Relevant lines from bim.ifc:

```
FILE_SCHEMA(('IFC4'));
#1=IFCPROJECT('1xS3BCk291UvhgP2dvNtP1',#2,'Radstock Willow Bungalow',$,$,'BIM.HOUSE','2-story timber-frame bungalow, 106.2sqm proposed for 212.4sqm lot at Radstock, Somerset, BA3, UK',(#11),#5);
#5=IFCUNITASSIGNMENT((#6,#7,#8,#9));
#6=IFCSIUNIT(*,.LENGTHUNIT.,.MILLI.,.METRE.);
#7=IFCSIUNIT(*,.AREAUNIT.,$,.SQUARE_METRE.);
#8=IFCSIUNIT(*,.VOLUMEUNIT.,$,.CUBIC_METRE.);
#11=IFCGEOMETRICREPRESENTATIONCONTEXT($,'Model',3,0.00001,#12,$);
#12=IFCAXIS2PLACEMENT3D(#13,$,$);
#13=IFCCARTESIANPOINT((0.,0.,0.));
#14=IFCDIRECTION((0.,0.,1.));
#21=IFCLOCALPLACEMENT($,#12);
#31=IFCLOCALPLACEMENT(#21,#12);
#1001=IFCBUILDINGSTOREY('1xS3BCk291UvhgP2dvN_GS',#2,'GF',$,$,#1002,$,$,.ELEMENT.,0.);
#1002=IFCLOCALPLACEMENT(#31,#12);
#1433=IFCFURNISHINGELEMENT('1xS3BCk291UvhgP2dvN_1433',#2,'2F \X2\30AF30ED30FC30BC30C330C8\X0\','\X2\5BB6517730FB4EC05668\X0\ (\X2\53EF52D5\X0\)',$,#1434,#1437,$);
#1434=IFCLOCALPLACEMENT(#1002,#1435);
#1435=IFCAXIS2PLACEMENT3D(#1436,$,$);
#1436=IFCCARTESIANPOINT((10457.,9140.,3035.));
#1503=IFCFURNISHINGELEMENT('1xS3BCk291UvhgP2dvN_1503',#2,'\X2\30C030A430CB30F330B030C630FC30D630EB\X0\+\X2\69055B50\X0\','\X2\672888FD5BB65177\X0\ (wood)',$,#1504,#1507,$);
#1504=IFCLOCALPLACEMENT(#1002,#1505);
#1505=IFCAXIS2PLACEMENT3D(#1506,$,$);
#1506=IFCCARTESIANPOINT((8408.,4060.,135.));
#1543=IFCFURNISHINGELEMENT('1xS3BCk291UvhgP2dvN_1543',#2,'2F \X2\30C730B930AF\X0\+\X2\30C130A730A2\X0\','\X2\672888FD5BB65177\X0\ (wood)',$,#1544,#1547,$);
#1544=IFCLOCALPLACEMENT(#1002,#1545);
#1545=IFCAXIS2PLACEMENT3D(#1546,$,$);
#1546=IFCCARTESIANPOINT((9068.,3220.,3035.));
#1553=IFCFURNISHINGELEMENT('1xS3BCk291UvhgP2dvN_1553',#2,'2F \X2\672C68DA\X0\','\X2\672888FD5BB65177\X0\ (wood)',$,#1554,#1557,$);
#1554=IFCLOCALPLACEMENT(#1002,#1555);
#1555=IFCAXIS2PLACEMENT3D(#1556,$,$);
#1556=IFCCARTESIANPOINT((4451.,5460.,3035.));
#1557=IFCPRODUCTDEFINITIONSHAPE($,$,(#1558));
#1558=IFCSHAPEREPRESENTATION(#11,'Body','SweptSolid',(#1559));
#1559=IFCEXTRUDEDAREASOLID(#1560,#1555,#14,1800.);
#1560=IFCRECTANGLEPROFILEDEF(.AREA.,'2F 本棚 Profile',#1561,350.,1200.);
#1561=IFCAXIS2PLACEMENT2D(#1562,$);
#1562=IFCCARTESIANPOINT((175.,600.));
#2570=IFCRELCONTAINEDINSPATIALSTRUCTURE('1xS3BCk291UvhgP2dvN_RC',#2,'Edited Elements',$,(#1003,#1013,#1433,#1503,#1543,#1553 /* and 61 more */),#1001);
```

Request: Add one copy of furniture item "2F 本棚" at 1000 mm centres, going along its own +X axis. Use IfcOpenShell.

```python
import ifcopenshell
import ifcopenshell.api.geometry
import ifcopenshell.api.root
import ifcopenshell.util.element
import ifcopenshell.util.placement

model = ifcopenshell.open("bim.ifc")


def reuse_history(source, copy):
    """copy_class also copies each property set's owner history, people and application; keep the originals."""
    for rel in copy.IsDefinedBy:
        if rel.is_a("IfcRelDefinesByProperties") and (history := rel.RelatingPropertyDefinition.OwnerHistory):
            rel.RelatingPropertyDefinition.OwnerHistory = source.OwnerHistory
            ifcopenshell.util.element.remove_deep2(model, history)


source = model.by_id(1553)
base = ifcopenshell.util.placement.get_local_placement(source.ObjectPlacement)
step = base[:3, 0] * 1000.0

for i in range(1, 2):
    copy = ifcopenshell.api.root.copy_class(model, product=source)
    copy.Representation = ifcopenshell.util.element.copy_deep(
        model, source.Representation, exclude=["IfcGeometricRepresentationContext", "IfcRepresentationMap"]
    )
    reuse_history(source, copy)
    matrix = base.copy()
    matrix[:3, 3] += i * step
    print("added at", matrix[:3, 3].round(3) + 0.0)
    ifcopenshell.api.geometry.edit_object_placement(model, product=copy, matrix=matrix, is_si=False)

model.write("bim_edited.ifc")
```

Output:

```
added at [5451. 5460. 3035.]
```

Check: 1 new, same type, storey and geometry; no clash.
